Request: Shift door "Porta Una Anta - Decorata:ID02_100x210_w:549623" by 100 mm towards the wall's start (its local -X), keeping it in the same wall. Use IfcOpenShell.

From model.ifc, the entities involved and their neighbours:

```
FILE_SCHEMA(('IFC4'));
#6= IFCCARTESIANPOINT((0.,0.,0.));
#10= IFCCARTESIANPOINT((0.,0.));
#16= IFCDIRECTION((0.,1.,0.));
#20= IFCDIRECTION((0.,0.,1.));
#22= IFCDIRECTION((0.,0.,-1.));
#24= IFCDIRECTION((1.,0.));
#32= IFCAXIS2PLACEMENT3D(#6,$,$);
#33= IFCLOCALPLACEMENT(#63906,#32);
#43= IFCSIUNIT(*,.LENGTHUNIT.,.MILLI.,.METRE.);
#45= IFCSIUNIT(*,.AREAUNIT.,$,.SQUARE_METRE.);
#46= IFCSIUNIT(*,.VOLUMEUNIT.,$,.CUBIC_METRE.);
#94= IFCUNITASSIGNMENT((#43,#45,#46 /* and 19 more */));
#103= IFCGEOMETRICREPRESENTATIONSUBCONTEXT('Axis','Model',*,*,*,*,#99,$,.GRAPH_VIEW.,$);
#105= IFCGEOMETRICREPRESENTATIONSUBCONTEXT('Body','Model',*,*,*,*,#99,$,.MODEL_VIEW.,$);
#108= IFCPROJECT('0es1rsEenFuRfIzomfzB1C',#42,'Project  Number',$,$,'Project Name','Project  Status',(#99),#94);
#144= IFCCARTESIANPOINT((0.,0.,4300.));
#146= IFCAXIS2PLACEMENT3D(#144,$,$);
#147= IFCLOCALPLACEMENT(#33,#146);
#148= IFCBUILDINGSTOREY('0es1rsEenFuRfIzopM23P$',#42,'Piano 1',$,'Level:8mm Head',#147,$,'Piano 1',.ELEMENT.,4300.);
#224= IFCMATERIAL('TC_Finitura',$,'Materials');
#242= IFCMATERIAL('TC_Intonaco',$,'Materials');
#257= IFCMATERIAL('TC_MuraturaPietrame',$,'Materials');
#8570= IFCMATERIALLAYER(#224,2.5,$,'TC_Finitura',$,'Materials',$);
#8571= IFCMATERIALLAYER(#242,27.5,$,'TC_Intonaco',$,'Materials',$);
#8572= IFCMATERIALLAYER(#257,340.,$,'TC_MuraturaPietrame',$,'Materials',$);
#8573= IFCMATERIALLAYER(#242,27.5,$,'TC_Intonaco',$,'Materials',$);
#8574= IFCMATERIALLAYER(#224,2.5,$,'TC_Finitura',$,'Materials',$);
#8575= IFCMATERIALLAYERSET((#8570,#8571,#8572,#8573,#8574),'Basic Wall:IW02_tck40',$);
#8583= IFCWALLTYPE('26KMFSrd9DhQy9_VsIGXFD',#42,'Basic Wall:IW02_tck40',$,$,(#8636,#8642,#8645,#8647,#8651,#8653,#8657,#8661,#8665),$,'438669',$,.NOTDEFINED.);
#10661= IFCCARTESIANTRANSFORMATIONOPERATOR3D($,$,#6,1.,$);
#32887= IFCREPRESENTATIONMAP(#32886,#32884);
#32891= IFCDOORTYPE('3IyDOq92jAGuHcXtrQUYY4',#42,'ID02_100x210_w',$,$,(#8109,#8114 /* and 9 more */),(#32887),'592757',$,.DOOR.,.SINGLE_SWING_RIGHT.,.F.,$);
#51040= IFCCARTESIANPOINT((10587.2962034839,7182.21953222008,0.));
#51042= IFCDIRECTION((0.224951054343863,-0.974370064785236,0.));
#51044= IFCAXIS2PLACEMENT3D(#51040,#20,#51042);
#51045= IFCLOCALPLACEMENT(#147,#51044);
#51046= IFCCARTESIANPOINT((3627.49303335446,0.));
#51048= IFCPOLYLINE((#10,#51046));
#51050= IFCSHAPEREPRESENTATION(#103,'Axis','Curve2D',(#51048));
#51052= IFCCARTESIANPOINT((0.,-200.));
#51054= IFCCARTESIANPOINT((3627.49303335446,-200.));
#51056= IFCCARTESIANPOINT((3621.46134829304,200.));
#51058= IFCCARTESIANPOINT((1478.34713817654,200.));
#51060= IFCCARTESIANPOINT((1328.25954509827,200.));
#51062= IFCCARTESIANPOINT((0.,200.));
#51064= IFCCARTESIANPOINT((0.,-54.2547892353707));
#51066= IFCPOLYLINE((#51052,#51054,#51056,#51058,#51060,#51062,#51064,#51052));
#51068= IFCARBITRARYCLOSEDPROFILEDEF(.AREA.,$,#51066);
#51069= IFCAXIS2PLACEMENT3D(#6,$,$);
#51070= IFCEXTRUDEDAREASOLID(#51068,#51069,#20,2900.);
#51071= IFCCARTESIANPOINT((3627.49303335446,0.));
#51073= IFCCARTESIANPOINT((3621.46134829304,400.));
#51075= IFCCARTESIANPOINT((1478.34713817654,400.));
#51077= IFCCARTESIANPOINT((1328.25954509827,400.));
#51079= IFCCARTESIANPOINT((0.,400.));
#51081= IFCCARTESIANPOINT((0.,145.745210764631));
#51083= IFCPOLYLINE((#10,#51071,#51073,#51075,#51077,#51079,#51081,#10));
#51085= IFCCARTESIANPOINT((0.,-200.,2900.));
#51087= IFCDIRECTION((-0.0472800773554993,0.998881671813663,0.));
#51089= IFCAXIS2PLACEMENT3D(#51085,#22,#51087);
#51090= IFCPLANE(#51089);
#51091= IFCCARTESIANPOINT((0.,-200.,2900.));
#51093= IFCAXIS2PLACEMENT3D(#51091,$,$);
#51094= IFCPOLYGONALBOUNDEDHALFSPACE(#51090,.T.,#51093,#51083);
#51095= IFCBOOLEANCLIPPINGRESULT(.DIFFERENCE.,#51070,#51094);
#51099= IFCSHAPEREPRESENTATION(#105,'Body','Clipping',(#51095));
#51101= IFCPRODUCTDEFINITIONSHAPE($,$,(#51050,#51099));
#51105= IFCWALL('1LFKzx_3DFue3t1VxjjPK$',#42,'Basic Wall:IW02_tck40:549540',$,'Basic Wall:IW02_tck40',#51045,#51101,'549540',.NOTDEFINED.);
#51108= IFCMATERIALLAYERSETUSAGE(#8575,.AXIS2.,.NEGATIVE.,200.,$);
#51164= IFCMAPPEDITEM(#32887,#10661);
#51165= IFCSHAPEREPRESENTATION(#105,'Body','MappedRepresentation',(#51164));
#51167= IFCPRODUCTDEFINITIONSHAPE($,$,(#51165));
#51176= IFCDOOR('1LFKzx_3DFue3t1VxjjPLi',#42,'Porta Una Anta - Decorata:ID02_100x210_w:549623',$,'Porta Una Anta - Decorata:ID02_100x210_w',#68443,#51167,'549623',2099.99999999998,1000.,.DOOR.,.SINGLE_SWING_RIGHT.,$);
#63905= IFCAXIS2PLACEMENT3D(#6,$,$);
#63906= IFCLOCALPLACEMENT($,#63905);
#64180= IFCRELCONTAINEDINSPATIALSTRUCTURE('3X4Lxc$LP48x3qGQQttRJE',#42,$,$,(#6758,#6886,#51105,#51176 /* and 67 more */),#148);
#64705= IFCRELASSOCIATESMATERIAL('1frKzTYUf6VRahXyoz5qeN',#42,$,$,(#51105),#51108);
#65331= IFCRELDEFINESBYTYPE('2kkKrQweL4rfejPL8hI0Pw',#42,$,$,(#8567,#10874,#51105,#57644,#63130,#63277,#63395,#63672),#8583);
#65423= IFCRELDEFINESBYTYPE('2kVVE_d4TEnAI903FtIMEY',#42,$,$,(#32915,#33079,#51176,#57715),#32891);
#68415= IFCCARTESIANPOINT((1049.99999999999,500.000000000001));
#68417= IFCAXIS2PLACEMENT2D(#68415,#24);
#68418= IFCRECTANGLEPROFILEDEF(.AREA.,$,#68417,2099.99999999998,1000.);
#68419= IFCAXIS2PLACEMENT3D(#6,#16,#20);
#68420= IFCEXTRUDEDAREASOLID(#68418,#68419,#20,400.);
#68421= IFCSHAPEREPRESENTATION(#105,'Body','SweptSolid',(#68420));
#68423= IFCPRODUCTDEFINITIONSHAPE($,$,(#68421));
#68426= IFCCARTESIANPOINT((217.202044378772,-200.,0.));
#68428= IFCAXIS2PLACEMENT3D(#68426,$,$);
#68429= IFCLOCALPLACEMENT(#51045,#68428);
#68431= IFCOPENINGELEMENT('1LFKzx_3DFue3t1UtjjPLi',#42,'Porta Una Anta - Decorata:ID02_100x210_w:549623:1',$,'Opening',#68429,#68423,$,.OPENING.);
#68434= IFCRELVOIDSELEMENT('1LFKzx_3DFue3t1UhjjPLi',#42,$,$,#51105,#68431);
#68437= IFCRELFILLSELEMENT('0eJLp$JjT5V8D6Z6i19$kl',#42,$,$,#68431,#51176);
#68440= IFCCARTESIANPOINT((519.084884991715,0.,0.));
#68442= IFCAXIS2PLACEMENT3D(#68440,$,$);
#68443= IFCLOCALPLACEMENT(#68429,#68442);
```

```python
import ifcopenshell
import ifcopenshell.api.geometry
import ifcopenshell.util.placement
import ifcopenshell.util.unit

model = ifcopenshell.open("model.ifc")
unit_scale = ifcopenshell.util.unit.calculate_unit_scale(model)

door = model.by_guid("1LFKzx_3DFue3t1VxjjPLi")
opening = door.FillsVoids[0].RelatingOpeningElement
wall = opening.VoidsElements[0].RelatingBuildingElement

wall_matrix = ifcopenshell.util.placement.get_local_placement(wall.ObjectPlacement)
shift = wall_matrix[:3, 0] * -0.1 / unit_scale
before = ifcopenshell.util.placement.get_local_placement(door.ObjectPlacement)[:3, 3].copy()

# The door is placed relative to its opening, so it follows when the opening moves.
matrix = ifcopenshell.util.placement.get_local_placement(opening.ObjectPlacement)
matrix[:3, 3] += shift
ifcopenshell.api.geometry.edit_object_placement(
    model, product=opening, matrix=matrix, is_si=False, should_transform_children=True
)

after = ifcopenshell.util.placement.get_local_placement(door.ObjectPlacement)[:3, 3]
print("door moved by", (after - before).round(3) + 0.0)

model.write("model_edited.ifc")
```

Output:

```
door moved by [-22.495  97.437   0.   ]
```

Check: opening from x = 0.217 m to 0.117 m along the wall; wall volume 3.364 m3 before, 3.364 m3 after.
